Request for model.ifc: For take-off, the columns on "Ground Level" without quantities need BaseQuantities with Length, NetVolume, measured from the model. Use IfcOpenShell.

First a look at what the model holds.

```python
import ifcopenshell
import ifcopenshell.util.element
import ifcopenshell.util.unit

model = ifcopenshell.open("model.ifc")
print(model.schema)
for unit_type in ("LENGTHUNIT", "AREAUNIT", "VOLUMEUNIT"):
    print(unit_type, ifcopenshell.util.unit.calculate_unit_scale(model, unit_type))
storey = next(s for s in model.by_type("IfcBuildingStorey") if s.Name == "Ground Level")
columns = [e for e in ifcopenshell.util.element.get_decomposition(storey) if e.is_a("IfcColumn")]
for e in sorted(columns, key=lambda e: e.id()):
    print(e.id(), e.is_a(), e.Name, list(ifcopenshell.util.element.get_psets(e, qtos_only=True)), sep=" | ")
```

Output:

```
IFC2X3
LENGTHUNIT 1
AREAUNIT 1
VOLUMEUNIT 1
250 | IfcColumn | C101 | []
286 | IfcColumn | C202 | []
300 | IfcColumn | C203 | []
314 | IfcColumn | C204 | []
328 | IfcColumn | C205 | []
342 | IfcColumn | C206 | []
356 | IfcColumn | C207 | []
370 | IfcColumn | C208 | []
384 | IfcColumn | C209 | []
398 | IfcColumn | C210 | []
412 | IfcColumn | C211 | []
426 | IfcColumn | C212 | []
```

```python
import ifcopenshell
import ifcopenshell.api.pset
import ifcopenshell.geom
import ifcopenshell.util.element
import ifcopenshell.util.shape
import ifcopenshell.util.unit

model = ifcopenshell.open("model.ifc")
unit_scale = ifcopenshell.util.unit.calculate_unit_scale(model)
volume_scale = ifcopenshell.util.unit.calculate_unit_scale(model, "VOLUMEUNIT")
settings = ifcopenshell.geom.settings()

storey = next(s for s in model.by_type("IfcBuildingStorey") if s.Name == "Ground Level")
columns = [e for e in ifcopenshell.util.element.get_decomposition(storey) if e.is_a("IfcColumn")]

for e in sorted(columns, key=lambda e: e.id()):
    if ifcopenshell.util.element.get_psets(e, qtos_only=True, should_inherit=False):
        continue
    # Geometry comes back in metres, in the element's own axes.
    shape = ifcopenshell.geom.create_shape(settings, e)
    values = {
        "Length": ifcopenshell.util.shape.get_z(shape.geometry) / unit_scale,
        "NetVolume": ifcopenshell.util.shape.get_volume(shape.geometry) / volume_scale,
    }
    qto = ifcopenshell.api.pset.add_qto(model, product=e, name="BaseQuantities")
    ifcopenshell.api.pset.edit_qto(model, qto=qto, properties=values)
    print(e.id(), {k: round(v, 3) for k, v in values.items()})

model.write("model_edited.ifc")
```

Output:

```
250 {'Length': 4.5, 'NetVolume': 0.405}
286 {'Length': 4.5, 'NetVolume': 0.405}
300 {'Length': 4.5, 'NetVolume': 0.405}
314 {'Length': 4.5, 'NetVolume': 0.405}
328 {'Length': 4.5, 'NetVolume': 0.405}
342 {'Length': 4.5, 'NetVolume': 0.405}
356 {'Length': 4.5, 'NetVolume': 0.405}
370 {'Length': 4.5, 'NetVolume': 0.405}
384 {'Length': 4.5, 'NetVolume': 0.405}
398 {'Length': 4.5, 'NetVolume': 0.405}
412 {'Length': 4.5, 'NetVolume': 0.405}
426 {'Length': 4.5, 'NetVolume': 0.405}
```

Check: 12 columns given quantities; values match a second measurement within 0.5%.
